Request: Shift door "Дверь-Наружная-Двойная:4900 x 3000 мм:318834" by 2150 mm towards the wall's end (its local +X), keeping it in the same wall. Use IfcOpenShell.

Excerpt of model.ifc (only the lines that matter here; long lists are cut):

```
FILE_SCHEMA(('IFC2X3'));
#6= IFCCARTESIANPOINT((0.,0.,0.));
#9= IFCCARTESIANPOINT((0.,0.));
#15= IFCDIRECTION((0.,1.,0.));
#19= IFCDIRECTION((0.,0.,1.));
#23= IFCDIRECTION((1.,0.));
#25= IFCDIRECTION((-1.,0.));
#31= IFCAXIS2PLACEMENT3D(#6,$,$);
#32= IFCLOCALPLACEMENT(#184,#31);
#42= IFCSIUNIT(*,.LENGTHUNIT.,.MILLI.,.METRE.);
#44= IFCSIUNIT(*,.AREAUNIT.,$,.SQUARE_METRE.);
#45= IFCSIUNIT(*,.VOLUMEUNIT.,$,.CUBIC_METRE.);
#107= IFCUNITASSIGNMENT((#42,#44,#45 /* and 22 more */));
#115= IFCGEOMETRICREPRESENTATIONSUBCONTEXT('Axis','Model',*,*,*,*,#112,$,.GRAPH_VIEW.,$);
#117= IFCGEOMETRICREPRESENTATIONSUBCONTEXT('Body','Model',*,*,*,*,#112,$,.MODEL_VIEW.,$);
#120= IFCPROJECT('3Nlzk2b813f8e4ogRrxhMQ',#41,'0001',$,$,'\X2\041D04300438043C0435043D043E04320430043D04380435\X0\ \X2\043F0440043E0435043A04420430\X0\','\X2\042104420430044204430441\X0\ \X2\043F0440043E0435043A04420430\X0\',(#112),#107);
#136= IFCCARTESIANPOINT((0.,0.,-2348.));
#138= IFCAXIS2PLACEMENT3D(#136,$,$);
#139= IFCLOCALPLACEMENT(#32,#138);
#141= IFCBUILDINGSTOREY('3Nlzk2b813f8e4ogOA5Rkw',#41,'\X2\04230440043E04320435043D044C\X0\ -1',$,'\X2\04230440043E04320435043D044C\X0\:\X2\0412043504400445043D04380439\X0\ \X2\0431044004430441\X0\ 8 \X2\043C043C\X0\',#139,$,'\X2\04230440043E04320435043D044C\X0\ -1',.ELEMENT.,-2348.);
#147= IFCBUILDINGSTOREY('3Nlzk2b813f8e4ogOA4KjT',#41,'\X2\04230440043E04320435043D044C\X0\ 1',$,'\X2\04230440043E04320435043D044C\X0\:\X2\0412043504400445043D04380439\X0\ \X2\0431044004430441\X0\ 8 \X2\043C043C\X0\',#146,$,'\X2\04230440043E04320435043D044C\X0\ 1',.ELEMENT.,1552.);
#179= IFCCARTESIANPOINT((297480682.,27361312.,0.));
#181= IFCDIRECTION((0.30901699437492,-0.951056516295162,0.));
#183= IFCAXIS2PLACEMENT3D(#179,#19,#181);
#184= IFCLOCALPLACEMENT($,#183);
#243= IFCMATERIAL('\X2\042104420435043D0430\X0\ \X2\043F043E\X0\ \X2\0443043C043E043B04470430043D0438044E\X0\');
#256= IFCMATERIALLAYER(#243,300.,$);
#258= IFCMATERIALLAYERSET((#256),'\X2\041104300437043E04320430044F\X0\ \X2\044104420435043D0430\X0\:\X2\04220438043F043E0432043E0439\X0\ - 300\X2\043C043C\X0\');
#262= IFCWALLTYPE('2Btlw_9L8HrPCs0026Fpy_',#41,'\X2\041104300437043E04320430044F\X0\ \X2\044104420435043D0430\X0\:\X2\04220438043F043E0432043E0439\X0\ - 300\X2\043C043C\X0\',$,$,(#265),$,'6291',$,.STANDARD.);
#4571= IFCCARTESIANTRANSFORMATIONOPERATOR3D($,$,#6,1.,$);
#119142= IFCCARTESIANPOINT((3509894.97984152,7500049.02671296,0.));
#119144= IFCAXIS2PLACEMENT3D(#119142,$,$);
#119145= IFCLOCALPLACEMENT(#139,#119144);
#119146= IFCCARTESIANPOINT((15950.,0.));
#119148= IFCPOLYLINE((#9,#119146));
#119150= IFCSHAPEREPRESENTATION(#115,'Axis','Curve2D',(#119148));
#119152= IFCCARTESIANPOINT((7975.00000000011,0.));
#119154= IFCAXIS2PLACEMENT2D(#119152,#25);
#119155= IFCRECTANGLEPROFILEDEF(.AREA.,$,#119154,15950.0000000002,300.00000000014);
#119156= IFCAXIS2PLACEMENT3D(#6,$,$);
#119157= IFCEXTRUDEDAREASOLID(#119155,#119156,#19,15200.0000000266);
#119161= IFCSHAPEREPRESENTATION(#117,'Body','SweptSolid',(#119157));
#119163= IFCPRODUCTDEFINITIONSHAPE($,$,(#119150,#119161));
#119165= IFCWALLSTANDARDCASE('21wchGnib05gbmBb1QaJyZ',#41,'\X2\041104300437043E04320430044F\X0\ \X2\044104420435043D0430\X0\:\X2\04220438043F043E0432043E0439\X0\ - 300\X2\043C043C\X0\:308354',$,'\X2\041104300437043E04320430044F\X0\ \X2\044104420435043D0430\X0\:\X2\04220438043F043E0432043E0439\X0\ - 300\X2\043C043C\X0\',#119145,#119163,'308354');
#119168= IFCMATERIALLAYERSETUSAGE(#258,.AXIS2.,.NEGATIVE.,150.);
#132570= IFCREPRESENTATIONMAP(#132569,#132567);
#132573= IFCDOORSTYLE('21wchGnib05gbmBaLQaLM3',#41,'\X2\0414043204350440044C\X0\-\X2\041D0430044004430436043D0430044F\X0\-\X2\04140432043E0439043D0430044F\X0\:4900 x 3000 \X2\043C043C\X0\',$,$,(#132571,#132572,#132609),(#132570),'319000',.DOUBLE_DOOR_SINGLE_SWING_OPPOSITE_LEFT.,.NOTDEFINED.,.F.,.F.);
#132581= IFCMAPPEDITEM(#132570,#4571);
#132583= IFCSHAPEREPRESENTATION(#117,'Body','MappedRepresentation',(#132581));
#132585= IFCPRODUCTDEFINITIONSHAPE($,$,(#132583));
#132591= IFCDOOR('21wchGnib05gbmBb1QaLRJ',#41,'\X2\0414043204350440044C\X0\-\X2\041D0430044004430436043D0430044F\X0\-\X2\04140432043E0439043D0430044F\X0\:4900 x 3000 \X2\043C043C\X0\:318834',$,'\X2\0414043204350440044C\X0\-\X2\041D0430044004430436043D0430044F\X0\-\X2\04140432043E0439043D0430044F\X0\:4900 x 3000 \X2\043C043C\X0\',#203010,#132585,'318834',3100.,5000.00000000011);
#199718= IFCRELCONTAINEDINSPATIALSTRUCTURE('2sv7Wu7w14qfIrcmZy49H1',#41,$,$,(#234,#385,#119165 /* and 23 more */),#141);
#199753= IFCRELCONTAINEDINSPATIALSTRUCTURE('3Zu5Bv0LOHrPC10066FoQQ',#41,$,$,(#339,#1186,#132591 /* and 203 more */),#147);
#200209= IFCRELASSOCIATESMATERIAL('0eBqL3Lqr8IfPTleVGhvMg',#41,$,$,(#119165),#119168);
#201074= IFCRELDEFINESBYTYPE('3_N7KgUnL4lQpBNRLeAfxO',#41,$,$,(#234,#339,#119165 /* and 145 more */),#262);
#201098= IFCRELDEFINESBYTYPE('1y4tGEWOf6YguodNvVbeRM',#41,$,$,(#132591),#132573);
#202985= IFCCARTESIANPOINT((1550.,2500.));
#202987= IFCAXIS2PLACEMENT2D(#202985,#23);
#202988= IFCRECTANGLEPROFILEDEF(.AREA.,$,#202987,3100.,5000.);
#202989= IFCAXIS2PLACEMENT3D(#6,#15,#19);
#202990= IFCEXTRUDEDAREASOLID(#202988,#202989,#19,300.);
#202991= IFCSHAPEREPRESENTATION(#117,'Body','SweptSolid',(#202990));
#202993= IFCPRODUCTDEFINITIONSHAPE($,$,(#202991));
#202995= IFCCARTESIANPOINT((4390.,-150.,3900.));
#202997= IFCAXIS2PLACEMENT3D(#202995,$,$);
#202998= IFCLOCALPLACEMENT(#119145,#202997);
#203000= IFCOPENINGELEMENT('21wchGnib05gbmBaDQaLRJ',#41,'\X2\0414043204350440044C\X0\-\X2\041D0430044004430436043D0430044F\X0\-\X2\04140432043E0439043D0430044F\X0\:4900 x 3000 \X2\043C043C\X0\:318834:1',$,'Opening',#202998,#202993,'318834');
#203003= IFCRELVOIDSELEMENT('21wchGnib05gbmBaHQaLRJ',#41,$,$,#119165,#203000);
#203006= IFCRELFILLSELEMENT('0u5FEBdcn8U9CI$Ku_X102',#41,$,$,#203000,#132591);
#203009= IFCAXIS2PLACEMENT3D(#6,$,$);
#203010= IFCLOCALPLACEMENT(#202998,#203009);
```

```python
import ifcopenshell
import ifcopenshell.api.geometry
import ifcopenshell.util.placement
import ifcopenshell.util.unit

model = ifcopenshell.open("model.ifc")
unit_scale = ifcopenshell.util.unit.calculate_unit_scale(model)

door = model.by_id(132591)
opening = door.FillsVoids[0].RelatingOpeningElement
wall = opening.VoidsElements[0].RelatingBuildingElement

wall_matrix = ifcopenshell.util.placement.get_local_placement(wall.ObjectPlacement)
shift = wall_matrix[:3, 0] * 2.15 / unit_scale
before = ifcopenshell.util.placement.get_local_placement(door.ObjectPlacement)[:3, 3].copy()

# The door is placed relative to its opening, so it follows when the opening moves.
matrix = ifcopenshell.util.placement.get_local_placement(opening.ObjectPlacement)
matrix[:3, 3] += shift
ifcopenshell.api.geometry.edit_object_placement(
    model, product=opening, matrix=matrix, is_si=False, should_transform_children=True
)

after = ifcopenshell.util.placement.get_local_placement(door.ObjectPlacement)[:3, 3]
print("door moved by", (after - before).round(3) + 0.0)

model.write("model-out.ifc")
```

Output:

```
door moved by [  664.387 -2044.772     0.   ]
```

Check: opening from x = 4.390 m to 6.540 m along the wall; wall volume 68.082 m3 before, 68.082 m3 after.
